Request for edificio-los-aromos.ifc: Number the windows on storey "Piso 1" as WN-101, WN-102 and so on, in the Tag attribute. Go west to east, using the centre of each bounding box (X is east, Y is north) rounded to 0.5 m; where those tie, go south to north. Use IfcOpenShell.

First a look at what the model holds.

```python
import ifcopenshell
import ifcopenshell.util.element
import ifcopenshell.util.placement

model = ifcopenshell.open("edificio-los-aromos.ifc")
print(model.schema)
storey = next(s for s in model.by_type("IfcBuildingStorey") if s.Name == "Piso 1")
windows = [e for e in ifcopenshell.util.element.get_decomposition(storey) if e.is_a("IfcWindow")]
for e in sorted(windows, key=lambda e: e.id()):
    origin = ifcopenshell.util.placement.get_local_placement(e.ObjectPlacement)[:3, 3]
    print(e.id(), e.Tag, e.Name, origin.round(2) + 0.0, sep=" | ")
```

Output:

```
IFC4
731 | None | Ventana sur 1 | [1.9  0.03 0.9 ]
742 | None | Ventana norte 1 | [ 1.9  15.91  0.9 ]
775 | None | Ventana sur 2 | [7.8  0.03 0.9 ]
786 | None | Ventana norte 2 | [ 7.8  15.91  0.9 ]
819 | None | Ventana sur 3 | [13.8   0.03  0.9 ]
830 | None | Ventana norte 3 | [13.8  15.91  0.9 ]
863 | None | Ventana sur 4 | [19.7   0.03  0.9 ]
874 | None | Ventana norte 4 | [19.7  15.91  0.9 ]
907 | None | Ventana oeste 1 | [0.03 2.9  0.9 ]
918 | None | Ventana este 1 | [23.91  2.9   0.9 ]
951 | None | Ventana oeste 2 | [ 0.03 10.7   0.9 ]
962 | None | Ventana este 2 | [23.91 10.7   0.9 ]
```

```python
import ifcopenshell
import ifcopenshell.geom
import ifcopenshell.util.element
import ifcopenshell.util.shape

model = ifcopenshell.open("edificio-los-aromos.ifc")
settings = ifcopenshell.geom.settings()
settings.set("use-world-coords", True)


def centre(element):
    shape = ifcopenshell.geom.create_shape(settings, element)
    return ifcopenshell.util.shape.get_bbox_centroid(shape.geometry)


storey = next(s for s in model.by_type("IfcBuildingStorey") if s.Name == "Piso 1")
windows = [e for e in ifcopenshell.util.element.get_decomposition(storey) if e.is_a("IfcWindow")]

# Insertion points can sit at a corner or the storey origin, so sort by the geometry (in metres).
centres = {e: centre(e) for e in windows}
windows.sort(key=lambda e: (round(centres[e][0] / 0.5), centres[e][1]))

for i, e in enumerate(windows, start=1):
    number = f"WN-1{i:02d}"
    e.Tag = number
    print(e.id(), number)

model.write("edificio-los-aromos_updated.ifc")
```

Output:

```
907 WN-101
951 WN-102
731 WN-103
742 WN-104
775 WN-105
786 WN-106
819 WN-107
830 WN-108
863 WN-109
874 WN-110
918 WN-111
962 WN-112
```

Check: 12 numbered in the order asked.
